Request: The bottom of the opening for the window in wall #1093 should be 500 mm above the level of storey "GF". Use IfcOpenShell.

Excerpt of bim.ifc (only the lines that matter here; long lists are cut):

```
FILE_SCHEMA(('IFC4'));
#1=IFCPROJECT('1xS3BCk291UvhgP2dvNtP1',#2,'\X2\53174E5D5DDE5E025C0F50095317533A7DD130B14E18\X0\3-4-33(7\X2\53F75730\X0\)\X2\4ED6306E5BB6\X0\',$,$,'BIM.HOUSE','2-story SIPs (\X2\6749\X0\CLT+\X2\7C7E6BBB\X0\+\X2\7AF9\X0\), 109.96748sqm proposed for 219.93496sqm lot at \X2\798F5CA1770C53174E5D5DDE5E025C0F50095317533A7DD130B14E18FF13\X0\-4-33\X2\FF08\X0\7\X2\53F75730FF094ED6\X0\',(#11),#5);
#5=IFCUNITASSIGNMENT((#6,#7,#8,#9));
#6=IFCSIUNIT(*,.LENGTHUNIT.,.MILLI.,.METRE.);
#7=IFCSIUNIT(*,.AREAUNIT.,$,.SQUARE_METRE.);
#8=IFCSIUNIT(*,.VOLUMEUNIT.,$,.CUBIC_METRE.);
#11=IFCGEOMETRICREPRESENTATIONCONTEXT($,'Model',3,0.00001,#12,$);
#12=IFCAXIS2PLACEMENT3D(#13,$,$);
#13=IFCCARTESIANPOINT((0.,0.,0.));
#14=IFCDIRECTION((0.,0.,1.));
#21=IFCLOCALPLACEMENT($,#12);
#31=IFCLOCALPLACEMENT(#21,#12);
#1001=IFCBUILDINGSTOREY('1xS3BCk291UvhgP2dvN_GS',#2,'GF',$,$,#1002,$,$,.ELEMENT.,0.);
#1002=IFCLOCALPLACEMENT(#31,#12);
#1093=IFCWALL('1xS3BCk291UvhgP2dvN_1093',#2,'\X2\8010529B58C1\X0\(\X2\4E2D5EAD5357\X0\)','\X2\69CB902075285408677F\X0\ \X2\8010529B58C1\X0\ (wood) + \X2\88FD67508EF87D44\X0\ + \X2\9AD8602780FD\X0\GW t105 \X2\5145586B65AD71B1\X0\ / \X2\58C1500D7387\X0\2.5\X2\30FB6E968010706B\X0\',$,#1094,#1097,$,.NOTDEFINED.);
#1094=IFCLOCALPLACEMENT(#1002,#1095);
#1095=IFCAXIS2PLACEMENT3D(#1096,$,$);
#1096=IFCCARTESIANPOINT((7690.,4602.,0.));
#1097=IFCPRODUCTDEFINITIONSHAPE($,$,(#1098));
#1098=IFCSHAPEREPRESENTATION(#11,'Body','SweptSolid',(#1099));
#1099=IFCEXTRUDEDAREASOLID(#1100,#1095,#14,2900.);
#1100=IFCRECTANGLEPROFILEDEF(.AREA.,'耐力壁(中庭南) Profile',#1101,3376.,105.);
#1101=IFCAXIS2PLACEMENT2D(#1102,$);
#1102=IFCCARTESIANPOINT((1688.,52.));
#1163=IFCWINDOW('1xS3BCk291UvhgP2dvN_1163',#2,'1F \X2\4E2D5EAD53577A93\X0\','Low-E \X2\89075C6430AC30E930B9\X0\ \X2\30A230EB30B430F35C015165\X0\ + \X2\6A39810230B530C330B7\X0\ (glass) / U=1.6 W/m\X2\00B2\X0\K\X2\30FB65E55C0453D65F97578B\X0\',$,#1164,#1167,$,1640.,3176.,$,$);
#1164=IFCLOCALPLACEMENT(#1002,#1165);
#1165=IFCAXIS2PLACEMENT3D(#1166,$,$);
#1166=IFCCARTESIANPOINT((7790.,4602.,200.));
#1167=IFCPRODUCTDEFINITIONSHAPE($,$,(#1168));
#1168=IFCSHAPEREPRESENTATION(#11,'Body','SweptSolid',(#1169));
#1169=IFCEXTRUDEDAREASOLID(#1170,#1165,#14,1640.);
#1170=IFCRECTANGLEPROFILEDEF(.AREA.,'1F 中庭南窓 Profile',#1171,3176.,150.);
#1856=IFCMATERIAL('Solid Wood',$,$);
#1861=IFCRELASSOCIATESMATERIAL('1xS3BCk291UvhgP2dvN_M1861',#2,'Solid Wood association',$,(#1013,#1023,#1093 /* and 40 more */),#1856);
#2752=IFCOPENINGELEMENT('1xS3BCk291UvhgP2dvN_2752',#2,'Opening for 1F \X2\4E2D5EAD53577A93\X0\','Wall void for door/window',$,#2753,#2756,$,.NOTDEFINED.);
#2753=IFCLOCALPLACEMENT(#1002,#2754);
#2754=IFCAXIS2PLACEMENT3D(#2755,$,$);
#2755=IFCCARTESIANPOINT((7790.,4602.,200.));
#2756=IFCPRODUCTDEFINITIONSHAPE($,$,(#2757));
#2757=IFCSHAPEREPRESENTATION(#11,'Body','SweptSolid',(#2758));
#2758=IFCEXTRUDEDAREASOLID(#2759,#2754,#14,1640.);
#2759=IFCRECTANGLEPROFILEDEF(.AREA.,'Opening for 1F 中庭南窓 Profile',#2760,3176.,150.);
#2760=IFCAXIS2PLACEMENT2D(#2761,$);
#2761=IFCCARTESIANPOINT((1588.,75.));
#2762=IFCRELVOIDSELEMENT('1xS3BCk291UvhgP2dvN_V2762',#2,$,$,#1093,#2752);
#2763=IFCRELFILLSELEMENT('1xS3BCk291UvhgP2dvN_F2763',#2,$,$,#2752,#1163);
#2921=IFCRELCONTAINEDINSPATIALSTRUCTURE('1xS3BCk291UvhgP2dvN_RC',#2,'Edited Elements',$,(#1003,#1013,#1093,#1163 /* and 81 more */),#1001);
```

```python
import numpy as np
import ifcopenshell
import ifcopenshell.api.geometry
import ifcopenshell.geom
import ifcopenshell.util.element
import ifcopenshell.util.placement
import ifcopenshell.util.shape
import ifcopenshell.util.unit

model = ifcopenshell.open("bim.ifc")
unit_scale = ifcopenshell.util.unit.calculate_unit_scale(model)

window = model.by_id(1163)
opening = window.FillsVoids[0].RelatingOpeningElement
storey = ifcopenshell.util.element.get_container(window, ifc_class="IfcBuildingStorey")
level = ifcopenshell.util.placement.get_local_placement(storey.ObjectPlacement)[2, 3]

# The opening's origin need not be at the sill, so measure its lowest point.
shape = ifcopenshell.geom.create_shape(ifcopenshell.geom.settings(), opening)
bottom = ifcopenshell.util.shape.get_shape_bottom_elevation(shape, shape.geometry) / unit_scale
dz = level + 0.5 / unit_scale - bottom

shift = np.array([0.0, 0.0, dz])
# The window is not placed relative to its opening, so move both.
for product in (opening, window):
    matrix = ifcopenshell.util.placement.get_local_placement(product.ObjectPlacement)
    matrix[:3, 3] += shift
    ifcopenshell.api.geometry.edit_object_placement(model, product=product, matrix=matrix, is_si=False)

print(f"moved by {dz * unit_scale:+.3f} m")

model.write("bim-out.ifc")
```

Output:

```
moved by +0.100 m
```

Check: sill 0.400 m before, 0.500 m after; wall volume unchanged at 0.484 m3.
